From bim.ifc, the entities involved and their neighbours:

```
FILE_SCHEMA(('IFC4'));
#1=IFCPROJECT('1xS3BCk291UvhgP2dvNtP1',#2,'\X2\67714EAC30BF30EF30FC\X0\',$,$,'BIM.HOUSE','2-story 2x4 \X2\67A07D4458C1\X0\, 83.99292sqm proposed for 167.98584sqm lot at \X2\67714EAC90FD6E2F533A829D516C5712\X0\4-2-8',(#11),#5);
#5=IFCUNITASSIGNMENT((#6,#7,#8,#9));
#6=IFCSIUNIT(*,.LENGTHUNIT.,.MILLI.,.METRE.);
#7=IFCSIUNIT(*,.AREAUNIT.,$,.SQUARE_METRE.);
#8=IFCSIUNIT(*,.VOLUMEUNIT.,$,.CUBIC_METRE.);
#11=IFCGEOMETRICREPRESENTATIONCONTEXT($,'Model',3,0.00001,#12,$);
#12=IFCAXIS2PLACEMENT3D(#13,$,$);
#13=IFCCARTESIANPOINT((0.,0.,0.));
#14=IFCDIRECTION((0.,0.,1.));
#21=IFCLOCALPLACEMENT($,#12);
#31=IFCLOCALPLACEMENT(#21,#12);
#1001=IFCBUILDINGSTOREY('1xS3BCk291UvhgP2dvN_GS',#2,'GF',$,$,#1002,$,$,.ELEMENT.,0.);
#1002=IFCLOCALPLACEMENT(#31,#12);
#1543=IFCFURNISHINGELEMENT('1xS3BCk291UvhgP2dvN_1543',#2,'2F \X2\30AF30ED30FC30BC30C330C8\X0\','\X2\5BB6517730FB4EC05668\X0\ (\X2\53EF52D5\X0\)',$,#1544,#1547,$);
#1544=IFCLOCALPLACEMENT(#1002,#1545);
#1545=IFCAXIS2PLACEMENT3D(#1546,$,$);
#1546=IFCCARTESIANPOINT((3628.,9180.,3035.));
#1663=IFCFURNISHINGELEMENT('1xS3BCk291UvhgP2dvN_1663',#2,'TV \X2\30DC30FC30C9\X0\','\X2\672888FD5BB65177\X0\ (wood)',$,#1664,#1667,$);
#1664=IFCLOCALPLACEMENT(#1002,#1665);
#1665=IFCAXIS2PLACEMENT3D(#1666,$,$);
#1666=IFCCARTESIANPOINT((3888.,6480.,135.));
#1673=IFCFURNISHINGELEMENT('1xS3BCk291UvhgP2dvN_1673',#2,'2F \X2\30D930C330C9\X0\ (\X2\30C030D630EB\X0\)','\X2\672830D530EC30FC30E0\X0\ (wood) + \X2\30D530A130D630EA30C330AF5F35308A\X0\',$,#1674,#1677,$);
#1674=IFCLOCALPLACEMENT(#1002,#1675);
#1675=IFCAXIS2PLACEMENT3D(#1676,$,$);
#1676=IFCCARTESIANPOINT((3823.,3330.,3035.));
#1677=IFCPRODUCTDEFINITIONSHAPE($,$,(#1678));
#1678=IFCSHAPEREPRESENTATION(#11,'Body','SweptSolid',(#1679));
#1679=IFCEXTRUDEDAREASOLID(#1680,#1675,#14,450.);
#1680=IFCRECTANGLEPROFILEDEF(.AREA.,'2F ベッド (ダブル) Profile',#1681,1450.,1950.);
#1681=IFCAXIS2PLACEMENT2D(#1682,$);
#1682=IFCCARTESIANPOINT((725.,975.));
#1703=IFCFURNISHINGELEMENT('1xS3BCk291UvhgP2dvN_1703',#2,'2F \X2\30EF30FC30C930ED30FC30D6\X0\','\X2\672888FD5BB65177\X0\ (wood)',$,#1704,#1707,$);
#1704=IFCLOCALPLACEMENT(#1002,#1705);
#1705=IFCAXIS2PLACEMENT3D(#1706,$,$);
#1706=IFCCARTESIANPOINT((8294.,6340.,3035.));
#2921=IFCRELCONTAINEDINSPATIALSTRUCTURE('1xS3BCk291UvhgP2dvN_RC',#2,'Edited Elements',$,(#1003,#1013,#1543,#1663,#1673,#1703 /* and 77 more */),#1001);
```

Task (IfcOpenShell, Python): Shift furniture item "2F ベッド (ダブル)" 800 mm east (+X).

```python
import ifcopenshell
import ifcopenshell.api.geometry
import ifcopenshell.util.placement
import ifcopenshell.util.unit

model = ifcopenshell.open("bim.ifc")
unit_scale = ifcopenshell.util.unit.calculate_unit_scale(model)

item = model.by_guid("1xS3BCk291UvhgP2dvN_1673")
matrix = ifcopenshell.util.placement.get_local_placement(item.ObjectPlacement)
matrix[0, 3] += 0.8 / unit_scale
ifcopenshell.api.geometry.edit_object_placement(model, product=item, matrix=matrix, is_si=False)

print(ifcopenshell.util.placement.get_local_placement(item.ObjectPlacement).round(3) + 0.0)

model.write("bim-out.ifc")
```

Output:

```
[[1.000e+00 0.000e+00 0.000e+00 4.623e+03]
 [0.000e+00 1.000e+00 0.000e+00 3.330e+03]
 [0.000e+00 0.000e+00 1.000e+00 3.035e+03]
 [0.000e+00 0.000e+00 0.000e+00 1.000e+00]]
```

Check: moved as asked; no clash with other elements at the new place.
